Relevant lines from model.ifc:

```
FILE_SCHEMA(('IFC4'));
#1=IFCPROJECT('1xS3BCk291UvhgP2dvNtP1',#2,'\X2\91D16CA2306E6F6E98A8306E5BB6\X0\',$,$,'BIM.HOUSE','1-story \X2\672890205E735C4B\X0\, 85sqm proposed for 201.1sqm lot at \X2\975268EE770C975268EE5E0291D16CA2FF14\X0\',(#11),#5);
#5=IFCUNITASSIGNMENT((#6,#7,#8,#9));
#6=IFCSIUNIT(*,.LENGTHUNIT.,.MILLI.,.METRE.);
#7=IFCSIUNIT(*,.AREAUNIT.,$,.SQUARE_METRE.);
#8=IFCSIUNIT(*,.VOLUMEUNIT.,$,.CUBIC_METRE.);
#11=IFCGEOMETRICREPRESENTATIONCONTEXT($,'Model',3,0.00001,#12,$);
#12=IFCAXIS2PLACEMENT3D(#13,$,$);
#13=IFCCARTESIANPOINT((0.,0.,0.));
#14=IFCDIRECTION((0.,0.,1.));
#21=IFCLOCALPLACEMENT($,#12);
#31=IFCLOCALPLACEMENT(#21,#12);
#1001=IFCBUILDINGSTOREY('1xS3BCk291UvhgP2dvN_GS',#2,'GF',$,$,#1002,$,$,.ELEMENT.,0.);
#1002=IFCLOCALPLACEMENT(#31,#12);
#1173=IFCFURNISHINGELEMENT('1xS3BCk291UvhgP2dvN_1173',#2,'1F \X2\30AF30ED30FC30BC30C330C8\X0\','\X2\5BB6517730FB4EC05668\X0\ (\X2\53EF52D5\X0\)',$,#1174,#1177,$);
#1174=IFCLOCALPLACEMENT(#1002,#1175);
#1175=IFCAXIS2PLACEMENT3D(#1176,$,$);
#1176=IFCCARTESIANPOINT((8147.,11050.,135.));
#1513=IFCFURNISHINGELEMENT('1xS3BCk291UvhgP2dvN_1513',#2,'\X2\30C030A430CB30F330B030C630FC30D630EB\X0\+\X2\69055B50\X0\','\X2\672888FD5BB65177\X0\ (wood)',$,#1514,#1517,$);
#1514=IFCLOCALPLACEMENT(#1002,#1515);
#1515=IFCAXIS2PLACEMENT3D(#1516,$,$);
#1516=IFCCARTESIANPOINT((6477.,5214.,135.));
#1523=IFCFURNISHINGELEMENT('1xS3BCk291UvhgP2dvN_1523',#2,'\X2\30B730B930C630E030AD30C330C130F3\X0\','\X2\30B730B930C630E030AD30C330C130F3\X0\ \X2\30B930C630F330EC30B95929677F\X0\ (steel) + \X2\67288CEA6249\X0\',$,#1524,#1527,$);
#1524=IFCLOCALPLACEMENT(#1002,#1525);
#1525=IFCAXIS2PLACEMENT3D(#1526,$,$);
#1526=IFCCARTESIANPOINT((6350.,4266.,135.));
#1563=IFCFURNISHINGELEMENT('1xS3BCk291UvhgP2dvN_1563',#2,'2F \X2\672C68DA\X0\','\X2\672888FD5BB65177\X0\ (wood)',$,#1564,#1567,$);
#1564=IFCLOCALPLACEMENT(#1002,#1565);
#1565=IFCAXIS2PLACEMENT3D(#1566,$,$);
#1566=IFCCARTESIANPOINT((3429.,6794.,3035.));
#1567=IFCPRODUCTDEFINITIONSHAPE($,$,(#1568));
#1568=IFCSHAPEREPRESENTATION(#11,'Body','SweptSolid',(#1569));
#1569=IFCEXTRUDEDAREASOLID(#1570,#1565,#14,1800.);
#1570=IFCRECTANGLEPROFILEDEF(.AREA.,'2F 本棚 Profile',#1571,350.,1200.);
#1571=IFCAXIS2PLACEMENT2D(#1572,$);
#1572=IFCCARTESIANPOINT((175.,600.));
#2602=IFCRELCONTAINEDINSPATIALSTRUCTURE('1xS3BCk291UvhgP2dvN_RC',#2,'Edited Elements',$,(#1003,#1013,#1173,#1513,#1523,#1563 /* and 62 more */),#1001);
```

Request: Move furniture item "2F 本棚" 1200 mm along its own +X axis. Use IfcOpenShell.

```python
import ifcopenshell
import ifcopenshell.api.geometry
import ifcopenshell.util.placement
import ifcopenshell.util.unit

model = ifcopenshell.open("model.ifc")
unit_scale = ifcopenshell.util.unit.calculate_unit_scale(model)

item = model.by_guid("1xS3BCk291UvhgP2dvN_1563")
matrix = ifcopenshell.util.placement.get_local_placement(item.ObjectPlacement)
matrix[:3, 3] += matrix[:3, 0] * 1.2 / unit_scale
ifcopenshell.api.geometry.edit_object_placement(model, product=item, matrix=matrix, is_si=False)

print(ifcopenshell.util.placement.get_local_placement(item.ObjectPlacement).round(3) + 0.0)

model.write("model_rev.ifc")
```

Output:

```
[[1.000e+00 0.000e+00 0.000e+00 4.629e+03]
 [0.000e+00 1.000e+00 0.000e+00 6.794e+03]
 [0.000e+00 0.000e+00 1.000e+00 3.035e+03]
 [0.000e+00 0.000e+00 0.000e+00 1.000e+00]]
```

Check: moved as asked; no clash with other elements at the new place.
